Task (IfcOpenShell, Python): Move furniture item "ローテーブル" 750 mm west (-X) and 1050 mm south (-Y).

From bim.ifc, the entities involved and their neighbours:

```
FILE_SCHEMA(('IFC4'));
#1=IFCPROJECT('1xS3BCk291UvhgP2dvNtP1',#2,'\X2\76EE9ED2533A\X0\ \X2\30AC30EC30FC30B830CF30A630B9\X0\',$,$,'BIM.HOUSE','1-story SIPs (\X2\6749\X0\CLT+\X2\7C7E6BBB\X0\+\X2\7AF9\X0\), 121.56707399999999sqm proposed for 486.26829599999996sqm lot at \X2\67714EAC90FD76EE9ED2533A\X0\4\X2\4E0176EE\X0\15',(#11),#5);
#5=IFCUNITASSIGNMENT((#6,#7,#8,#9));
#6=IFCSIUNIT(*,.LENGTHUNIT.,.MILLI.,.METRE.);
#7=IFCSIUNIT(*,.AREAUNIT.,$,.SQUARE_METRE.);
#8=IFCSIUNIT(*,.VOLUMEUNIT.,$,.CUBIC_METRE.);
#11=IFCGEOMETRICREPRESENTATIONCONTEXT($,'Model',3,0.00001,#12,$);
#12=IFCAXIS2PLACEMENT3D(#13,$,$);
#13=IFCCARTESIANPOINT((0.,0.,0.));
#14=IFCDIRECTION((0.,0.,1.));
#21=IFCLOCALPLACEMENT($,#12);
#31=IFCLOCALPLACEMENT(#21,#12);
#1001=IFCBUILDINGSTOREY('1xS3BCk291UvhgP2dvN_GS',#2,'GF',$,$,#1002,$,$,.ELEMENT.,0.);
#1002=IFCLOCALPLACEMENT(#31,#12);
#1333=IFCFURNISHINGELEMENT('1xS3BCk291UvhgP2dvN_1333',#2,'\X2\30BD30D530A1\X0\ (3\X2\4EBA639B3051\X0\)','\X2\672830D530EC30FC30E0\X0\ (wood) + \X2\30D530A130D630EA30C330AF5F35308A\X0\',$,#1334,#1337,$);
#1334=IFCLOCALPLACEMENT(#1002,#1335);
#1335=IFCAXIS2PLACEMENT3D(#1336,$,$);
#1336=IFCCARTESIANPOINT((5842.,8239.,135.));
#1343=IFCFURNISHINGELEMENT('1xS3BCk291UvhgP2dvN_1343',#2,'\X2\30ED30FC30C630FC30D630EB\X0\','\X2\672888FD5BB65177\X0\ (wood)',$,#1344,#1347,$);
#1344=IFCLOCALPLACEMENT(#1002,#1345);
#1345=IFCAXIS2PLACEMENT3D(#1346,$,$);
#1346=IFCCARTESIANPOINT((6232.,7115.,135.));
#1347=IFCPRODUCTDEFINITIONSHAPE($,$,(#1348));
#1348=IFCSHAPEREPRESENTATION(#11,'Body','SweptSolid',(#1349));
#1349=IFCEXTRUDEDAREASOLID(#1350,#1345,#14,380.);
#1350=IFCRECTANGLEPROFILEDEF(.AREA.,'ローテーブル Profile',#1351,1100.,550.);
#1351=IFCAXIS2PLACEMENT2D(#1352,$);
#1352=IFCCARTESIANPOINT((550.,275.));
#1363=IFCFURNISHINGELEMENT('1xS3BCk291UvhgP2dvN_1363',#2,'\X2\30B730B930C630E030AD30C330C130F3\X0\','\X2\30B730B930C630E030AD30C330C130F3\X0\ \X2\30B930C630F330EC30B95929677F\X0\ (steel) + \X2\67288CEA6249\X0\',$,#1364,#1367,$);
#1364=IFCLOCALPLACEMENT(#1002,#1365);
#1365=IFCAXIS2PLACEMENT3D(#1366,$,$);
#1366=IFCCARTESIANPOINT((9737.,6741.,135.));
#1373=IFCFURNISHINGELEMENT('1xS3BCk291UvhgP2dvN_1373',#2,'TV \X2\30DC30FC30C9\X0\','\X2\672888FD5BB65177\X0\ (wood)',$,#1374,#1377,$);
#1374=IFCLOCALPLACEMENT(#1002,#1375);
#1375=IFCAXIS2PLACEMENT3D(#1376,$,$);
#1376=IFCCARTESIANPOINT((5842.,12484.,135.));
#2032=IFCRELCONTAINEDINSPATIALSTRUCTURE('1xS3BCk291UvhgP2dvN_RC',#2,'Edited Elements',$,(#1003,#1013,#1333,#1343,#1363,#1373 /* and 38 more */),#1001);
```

```python
import ifcopenshell
import ifcopenshell.api.geometry
import ifcopenshell.util.placement
import ifcopenshell.util.unit

model = ifcopenshell.open("bim.ifc")
unit_scale = ifcopenshell.util.unit.calculate_unit_scale(model)

item = model.by_guid("1xS3BCk291UvhgP2dvN_1343")
matrix = ifcopenshell.util.placement.get_local_placement(item.ObjectPlacement)
matrix[0, 3] -= 0.75 / unit_scale
matrix[1, 3] -= 1.05 / unit_scale
ifcopenshell.api.geometry.edit_object_placement(model, product=item, matrix=matrix, is_si=False)

print(ifcopenshell.util.placement.get_local_placement(item.ObjectPlacement).round(3) + 0.0)

model.write("bim_v2.ifc")
```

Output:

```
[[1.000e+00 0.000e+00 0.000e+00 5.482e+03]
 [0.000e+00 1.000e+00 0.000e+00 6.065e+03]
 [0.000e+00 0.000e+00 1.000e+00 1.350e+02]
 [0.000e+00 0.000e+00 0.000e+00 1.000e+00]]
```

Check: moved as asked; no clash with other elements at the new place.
